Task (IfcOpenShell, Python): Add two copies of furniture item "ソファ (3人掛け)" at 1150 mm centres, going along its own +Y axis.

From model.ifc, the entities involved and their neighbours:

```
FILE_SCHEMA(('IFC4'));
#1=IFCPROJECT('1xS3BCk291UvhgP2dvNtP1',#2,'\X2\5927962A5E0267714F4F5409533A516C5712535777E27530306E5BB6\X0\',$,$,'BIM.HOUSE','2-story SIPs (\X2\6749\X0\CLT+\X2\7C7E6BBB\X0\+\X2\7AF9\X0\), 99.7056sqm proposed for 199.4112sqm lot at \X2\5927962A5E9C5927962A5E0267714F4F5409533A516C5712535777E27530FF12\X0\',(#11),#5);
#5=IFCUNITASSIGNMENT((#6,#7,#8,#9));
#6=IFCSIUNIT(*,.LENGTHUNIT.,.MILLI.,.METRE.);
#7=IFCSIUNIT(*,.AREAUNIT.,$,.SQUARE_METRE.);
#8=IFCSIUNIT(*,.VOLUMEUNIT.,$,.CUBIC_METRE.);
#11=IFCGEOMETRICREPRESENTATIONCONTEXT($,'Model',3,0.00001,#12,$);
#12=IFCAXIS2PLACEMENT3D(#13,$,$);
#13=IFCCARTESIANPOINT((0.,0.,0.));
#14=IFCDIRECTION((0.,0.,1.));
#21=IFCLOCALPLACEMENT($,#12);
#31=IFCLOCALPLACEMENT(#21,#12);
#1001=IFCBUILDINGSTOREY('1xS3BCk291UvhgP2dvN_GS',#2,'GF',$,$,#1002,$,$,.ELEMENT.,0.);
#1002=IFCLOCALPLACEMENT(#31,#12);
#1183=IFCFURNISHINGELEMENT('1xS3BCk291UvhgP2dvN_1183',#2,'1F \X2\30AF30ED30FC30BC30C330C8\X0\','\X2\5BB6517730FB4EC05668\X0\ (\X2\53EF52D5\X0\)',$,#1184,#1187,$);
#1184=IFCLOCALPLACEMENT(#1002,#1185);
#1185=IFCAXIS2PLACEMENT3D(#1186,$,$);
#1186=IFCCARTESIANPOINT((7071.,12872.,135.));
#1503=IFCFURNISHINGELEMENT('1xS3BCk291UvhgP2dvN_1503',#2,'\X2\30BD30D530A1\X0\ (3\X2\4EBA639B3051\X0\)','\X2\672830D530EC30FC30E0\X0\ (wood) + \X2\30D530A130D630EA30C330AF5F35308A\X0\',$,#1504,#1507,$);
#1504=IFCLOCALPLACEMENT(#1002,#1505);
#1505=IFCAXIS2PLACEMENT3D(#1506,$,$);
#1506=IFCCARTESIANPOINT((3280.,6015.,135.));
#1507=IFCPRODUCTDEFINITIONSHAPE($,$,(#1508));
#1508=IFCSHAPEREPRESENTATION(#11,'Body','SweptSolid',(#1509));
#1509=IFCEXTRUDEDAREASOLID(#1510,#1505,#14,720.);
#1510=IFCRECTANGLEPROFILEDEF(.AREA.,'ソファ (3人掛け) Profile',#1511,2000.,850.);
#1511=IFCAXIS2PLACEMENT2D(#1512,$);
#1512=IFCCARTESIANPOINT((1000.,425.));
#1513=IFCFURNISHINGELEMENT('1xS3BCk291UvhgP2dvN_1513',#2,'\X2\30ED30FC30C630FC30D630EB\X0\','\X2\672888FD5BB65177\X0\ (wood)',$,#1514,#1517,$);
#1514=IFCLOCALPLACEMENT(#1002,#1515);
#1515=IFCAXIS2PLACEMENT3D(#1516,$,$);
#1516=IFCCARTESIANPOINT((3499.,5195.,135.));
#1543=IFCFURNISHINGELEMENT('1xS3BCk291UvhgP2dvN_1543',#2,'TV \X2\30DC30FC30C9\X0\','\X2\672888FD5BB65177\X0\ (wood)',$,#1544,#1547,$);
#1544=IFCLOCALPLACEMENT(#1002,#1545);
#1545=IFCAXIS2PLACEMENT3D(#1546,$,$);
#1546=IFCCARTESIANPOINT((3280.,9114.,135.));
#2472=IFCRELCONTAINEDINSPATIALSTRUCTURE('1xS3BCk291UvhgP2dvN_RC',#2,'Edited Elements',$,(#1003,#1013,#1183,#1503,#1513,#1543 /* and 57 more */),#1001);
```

```python
import ifcopenshell
import ifcopenshell.api.geometry
import ifcopenshell.api.root
import ifcopenshell.util.element
import ifcopenshell.util.placement
import ifcopenshell.util.unit

model = ifcopenshell.open("model.ifc")
unit_scale = ifcopenshell.util.unit.calculate_unit_scale(model)


def reuse_history(source, copy):
    """copy_class also copies each property set's owner history, people and application; keep the originals."""
    for rel in copy.IsDefinedBy:
        if rel.is_a("IfcRelDefinesByProperties") and (history := rel.RelatingPropertyDefinition.OwnerHistory):
            rel.RelatingPropertyDefinition.OwnerHistory = source.OwnerHistory
            ifcopenshell.util.element.remove_deep2(model, history)


source = model.by_id(1503)
base = ifcopenshell.util.placement.get_local_placement(source.ObjectPlacement)
step = base[:3, 1] * 1.15 / unit_scale

for i in range(1, 3):
    copy = ifcopenshell.api.root.copy_class(model, product=source)
    copy.Representation = ifcopenshell.util.element.copy_deep(
        model, source.Representation, exclude=["IfcGeometricRepresentationContext", "IfcRepresentationMap"]
    )
    reuse_history(source, copy)
    matrix = base.copy()
    matrix[:3, 3] += i * step
    print("added at", matrix[:3, 3].round(3) + 0.0)
    ifcopenshell.api.geometry.edit_object_placement(model, product=copy, matrix=matrix, is_si=False)

model.write("model_rev.ifc")
```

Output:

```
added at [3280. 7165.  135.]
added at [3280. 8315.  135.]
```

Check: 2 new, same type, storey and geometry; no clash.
